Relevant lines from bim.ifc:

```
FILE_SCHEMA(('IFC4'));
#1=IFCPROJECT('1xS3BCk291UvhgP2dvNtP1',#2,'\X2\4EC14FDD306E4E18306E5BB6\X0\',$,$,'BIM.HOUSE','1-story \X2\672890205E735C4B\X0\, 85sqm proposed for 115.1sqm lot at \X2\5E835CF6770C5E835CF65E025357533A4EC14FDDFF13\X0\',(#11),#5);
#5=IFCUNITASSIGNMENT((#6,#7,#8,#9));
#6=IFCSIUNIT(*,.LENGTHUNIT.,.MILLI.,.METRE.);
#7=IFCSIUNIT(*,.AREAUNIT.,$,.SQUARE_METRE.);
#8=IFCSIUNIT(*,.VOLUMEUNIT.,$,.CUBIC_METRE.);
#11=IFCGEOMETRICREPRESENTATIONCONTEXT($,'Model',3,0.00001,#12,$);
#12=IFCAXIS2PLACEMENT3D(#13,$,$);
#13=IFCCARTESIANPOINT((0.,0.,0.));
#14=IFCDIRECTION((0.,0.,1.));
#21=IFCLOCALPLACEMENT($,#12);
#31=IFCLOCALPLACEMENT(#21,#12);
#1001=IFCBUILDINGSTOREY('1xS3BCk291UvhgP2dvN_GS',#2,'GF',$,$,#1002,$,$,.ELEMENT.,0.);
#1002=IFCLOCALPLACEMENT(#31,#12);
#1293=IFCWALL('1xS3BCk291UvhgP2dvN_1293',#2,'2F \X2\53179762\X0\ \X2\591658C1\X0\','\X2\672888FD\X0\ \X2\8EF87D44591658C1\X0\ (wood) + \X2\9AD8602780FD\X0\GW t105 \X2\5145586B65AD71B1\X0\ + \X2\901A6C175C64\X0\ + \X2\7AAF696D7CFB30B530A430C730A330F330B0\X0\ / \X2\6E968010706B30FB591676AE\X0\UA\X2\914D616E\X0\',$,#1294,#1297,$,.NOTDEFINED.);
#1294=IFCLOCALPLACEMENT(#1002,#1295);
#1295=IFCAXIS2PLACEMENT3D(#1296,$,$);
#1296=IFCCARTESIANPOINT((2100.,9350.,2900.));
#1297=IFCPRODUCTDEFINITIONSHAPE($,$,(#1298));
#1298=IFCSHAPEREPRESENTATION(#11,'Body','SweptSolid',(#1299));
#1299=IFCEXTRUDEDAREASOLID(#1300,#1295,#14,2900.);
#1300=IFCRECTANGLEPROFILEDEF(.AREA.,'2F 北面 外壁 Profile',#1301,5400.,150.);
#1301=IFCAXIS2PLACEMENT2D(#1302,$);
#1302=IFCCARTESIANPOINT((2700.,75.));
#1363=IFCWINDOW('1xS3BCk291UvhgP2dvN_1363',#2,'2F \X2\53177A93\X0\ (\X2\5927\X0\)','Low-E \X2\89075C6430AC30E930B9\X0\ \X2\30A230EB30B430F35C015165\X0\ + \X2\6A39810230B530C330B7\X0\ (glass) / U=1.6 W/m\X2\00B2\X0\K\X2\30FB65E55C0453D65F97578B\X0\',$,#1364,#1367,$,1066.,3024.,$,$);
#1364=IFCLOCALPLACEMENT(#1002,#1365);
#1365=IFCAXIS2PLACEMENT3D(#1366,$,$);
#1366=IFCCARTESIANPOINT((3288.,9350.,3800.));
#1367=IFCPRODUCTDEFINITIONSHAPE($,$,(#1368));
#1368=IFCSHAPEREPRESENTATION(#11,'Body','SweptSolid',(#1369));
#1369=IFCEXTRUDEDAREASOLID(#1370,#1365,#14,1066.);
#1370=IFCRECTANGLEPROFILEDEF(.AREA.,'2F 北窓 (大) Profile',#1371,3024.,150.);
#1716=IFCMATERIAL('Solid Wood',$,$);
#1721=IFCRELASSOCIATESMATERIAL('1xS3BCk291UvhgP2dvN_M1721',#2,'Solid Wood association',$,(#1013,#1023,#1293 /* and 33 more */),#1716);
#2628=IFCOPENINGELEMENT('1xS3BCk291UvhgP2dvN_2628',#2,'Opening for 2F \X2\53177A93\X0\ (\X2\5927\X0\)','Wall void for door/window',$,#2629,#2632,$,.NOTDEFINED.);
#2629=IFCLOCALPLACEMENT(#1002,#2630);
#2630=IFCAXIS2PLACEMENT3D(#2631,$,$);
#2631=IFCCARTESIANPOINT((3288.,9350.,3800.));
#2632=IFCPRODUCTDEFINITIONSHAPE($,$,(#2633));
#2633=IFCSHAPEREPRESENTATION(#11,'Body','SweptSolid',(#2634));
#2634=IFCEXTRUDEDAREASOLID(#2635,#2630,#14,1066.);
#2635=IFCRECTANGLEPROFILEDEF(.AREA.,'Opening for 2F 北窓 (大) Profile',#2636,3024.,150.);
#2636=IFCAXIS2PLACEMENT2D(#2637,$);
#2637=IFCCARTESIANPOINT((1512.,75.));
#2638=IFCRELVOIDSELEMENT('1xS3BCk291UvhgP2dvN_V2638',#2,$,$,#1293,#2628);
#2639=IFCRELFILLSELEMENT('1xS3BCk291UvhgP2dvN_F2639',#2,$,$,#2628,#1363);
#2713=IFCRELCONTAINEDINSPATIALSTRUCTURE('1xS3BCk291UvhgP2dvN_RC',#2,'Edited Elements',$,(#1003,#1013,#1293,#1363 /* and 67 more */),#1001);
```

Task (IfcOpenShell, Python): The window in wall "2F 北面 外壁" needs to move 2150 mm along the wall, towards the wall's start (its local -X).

```python
import ifcopenshell
import ifcopenshell.api.geometry
import ifcopenshell.util.placement

model = ifcopenshell.open("bim.ifc")

window = model.by_guid("1xS3BCk291UvhgP2dvN_1363")
opening = window.FillsVoids[0].RelatingOpeningElement
wall = opening.VoidsElements[0].RelatingBuildingElement

wall_matrix = ifcopenshell.util.placement.get_local_placement(wall.ObjectPlacement)
shift = wall_matrix[:3, 0] * -2150.0
before = ifcopenshell.util.placement.get_local_placement(window.ObjectPlacement)[:3, 3].copy()

# The window is not placed relative to its opening, so move both.
for product in (opening, window):
    matrix = ifcopenshell.util.placement.get_local_placement(product.ObjectPlacement)
    matrix[:3, 3] += shift
    ifcopenshell.api.geometry.edit_object_placement(model, product=product, matrix=matrix, is_si=False)

after = ifcopenshell.util.placement.get_local_placement(window.ObjectPlacement)[:3, 3]
print("window moved by", (after - before).round(3) + 0.0)

model.write("bim_edited.ifc")
```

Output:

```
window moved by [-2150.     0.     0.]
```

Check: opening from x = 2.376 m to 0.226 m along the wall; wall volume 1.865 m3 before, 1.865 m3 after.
